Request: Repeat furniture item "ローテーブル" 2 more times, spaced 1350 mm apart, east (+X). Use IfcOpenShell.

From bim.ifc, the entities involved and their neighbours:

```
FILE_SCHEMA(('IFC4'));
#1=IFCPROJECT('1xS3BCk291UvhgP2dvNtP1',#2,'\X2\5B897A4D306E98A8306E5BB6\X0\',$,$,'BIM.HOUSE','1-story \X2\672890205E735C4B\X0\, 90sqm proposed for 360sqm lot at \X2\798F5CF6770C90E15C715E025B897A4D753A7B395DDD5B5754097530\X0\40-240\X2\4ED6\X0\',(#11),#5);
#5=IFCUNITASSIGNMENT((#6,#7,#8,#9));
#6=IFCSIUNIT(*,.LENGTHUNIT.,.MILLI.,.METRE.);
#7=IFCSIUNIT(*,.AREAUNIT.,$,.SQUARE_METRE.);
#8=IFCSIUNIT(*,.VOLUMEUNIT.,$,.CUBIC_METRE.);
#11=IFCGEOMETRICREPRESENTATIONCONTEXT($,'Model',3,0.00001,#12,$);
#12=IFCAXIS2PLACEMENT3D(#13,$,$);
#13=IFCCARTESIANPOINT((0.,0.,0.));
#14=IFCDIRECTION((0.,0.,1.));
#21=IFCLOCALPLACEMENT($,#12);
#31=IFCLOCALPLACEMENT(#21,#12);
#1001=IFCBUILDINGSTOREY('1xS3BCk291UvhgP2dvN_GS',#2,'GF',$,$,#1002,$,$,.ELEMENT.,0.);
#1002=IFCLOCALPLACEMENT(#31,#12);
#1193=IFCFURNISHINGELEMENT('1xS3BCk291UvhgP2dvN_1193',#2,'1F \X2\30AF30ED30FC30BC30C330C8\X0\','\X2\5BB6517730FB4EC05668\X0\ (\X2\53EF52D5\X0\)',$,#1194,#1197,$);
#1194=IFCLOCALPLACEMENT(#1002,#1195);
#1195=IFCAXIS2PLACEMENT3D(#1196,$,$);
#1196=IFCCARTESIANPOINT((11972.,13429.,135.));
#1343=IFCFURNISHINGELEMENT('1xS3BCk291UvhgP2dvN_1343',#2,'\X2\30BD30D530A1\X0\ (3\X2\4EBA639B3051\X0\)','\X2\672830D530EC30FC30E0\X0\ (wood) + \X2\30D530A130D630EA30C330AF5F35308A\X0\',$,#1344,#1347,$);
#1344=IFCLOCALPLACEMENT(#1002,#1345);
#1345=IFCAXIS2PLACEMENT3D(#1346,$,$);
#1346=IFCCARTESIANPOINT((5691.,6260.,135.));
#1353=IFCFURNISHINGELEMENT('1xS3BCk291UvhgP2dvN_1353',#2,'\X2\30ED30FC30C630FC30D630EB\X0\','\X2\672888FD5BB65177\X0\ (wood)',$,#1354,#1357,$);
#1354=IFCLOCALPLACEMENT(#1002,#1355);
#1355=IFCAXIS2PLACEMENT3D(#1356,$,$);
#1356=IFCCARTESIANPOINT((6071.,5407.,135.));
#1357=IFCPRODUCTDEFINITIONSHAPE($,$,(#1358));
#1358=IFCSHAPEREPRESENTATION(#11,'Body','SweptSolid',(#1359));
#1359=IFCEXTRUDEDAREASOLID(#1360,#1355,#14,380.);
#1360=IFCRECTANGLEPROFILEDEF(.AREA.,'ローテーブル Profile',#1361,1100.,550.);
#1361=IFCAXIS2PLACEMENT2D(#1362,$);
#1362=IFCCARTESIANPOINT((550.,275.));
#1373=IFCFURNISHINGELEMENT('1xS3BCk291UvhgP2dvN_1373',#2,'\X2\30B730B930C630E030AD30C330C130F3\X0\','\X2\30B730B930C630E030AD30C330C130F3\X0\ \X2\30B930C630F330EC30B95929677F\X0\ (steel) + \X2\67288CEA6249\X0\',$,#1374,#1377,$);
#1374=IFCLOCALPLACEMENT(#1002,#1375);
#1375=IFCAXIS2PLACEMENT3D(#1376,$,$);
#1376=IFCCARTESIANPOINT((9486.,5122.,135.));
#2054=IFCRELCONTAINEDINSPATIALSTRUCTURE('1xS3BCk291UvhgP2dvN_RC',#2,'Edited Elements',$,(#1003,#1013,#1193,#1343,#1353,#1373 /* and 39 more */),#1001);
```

```python
import numpy as np
import ifcopenshell
import ifcopenshell.api.geometry
import ifcopenshell.api.root
import ifcopenshell.util.element
import ifcopenshell.util.placement

model = ifcopenshell.open("bim.ifc")


def reuse_history(source, copy):
    """copy_class also copies each property set's owner history, people and application; keep the originals."""
    for rel in copy.IsDefinedBy:
        if rel.is_a("IfcRelDefinesByProperties") and (history := rel.RelatingPropertyDefinition.OwnerHistory):
            rel.RelatingPropertyDefinition.OwnerHistory = source.OwnerHistory
            ifcopenshell.util.element.remove_deep2(model, history)


source = model.by_guid("1xS3BCk291UvhgP2dvN_1353")
base = ifcopenshell.util.placement.get_local_placement(source.ObjectPlacement)
step = np.array([1.0, 0.0, 0.0]) * 1350.0

for i in range(1, 3):
    copy = ifcopenshell.api.root.copy_class(model, product=source)
    copy.Representation = ifcopenshell.util.element.copy_deep(
        model, source.Representation, exclude=["IfcGeometricRepresentationContext", "IfcRepresentationMap"]
    )
    reuse_history(source, copy)
    matrix = base.copy()
    matrix[:3, 3] += i * step
    print("added at", matrix[:3, 3].round(3) + 0.0)
    ifcopenshell.api.geometry.edit_object_placement(model, product=copy, matrix=matrix, is_si=False)

model.write("bim_v2.ifc")
```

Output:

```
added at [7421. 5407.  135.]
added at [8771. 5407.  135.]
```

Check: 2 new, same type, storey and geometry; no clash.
